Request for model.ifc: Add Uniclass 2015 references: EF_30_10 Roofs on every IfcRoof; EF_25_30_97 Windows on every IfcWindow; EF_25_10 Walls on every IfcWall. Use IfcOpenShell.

First a look at what the model holds.

```python
import ifcopenshell

model = ifcopenshell.open("model.ifc")
print(model.schema)
print("classifications:", [c.Name for c in model.by_type("IfcClassification")])
for ifc_class in ("IfcDoor", "IfcRoof", "IfcStair", "IfcWall", "IfcWindow"):
    print(ifc_class, len(model.by_type(ifc_class)))
```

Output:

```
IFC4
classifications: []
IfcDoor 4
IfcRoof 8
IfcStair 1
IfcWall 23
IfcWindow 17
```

```python
import ifcopenshell
import ifcopenshell.api.classification

model = ifcopenshell.open("model.ifc")

system = ifcopenshell.api.classification.add_classification(model, classification="Uniclass 2015")

codes = {
    "IfcRoof": ("EF_30_10", "Roofs"),
    "IfcWindow": ("EF_25_30_97", "Windows"),
    "IfcWall": ("EF_25_10", "Walls"),
}
for ifc_class, (code, name) in codes.items():
    products = model.by_type(ifc_class)
    ifcopenshell.api.classification.add_reference(
        model, products=products, classification=system, identification=code, name=name
    )
    print(code, len(products))

model.write("model-out.ifc")
```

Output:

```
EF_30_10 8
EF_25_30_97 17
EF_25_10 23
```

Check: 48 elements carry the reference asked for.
